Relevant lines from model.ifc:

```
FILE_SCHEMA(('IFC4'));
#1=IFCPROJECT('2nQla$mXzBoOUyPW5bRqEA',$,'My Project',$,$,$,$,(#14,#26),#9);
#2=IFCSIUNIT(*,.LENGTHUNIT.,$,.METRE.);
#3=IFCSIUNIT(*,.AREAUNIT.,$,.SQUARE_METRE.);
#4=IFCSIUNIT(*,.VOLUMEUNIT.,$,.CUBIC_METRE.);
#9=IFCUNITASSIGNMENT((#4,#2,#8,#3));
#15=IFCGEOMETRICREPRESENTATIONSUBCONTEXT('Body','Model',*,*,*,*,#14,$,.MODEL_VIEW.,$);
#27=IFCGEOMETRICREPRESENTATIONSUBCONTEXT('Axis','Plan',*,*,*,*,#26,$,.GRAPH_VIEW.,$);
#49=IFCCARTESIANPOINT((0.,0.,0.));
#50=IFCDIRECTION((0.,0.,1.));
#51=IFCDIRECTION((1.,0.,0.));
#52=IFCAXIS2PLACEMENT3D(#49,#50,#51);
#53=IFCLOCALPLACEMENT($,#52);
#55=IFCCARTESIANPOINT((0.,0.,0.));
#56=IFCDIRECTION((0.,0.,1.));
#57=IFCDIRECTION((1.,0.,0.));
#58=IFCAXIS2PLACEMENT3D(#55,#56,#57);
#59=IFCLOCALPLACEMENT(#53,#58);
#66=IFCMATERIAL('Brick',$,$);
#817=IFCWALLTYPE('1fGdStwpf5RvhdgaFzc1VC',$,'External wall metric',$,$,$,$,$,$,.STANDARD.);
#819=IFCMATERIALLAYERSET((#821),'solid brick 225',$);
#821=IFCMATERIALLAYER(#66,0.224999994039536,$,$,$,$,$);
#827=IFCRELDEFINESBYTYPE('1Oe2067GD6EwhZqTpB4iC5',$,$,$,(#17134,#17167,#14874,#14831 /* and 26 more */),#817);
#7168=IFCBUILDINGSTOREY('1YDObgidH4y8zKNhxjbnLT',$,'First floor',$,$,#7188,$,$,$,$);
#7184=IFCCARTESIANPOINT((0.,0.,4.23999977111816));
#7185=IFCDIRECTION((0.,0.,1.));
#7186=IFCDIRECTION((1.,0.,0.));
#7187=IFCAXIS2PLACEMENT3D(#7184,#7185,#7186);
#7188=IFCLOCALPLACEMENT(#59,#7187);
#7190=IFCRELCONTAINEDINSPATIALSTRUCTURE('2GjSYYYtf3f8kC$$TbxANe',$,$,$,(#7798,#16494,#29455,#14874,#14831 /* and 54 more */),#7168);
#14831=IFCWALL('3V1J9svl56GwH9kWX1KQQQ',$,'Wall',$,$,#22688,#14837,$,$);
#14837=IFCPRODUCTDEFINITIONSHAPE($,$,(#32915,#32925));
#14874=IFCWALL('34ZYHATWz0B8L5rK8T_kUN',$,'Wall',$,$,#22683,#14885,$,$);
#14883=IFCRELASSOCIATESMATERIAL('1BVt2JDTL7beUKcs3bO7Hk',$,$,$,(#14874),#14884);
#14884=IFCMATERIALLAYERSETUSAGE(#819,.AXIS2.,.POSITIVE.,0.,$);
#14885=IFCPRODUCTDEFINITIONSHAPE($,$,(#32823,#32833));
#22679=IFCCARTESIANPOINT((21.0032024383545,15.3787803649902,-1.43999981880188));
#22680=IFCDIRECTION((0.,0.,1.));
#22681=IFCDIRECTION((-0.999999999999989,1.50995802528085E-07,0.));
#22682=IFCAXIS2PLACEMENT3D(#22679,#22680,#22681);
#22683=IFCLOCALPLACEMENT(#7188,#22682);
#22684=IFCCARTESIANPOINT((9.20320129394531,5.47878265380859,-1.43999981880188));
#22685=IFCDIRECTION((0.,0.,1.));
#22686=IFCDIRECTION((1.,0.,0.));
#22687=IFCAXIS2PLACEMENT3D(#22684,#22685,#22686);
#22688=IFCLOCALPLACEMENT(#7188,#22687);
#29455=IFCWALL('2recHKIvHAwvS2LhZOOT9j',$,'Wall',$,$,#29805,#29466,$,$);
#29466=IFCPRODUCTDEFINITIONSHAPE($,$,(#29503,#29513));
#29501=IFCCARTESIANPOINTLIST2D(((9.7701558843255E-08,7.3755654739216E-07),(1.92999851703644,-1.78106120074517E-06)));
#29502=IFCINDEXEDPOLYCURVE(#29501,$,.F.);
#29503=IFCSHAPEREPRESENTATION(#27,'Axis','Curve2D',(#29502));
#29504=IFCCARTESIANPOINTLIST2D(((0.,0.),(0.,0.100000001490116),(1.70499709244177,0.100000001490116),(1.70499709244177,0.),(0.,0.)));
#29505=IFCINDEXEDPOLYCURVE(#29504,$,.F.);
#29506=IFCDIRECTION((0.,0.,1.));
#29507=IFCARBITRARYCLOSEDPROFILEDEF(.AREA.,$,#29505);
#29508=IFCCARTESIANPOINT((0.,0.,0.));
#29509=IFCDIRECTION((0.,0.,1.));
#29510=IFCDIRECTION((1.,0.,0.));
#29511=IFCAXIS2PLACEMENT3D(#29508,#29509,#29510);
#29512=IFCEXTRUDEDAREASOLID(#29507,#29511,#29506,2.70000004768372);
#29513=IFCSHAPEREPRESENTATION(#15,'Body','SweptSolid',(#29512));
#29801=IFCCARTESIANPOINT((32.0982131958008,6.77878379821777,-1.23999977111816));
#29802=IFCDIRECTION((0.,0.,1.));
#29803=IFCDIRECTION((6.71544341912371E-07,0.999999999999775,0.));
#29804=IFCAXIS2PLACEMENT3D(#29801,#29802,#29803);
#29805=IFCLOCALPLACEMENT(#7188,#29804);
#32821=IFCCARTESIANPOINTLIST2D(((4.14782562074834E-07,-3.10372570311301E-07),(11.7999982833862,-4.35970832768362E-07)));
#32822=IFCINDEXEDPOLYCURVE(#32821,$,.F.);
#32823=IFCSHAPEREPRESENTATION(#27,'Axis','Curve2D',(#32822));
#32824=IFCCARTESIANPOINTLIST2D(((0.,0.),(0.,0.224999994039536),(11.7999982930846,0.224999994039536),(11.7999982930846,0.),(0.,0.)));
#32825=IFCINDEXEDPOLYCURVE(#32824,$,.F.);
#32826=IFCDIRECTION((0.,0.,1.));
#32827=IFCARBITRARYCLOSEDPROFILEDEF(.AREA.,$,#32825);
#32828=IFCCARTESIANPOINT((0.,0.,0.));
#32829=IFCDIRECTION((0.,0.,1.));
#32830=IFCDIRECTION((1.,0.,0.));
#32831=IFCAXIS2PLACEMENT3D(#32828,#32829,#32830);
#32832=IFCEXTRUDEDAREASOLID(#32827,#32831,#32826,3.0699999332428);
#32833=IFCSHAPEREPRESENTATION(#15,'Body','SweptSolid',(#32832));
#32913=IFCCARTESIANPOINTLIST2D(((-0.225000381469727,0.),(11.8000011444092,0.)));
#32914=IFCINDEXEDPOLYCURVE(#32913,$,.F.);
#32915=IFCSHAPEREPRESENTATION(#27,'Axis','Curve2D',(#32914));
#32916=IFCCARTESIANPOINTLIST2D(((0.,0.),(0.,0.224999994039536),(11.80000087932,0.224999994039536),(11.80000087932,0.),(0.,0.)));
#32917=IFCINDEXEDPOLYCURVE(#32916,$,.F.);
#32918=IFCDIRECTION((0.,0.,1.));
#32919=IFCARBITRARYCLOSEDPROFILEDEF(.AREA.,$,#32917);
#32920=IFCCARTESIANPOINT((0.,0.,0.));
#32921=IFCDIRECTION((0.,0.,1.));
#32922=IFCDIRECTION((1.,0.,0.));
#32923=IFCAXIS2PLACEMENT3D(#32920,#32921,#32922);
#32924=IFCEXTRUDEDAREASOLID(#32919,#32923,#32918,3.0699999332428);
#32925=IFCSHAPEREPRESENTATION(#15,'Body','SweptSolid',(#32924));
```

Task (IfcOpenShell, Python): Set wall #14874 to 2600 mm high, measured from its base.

```python
import ifcopenshell
import ifcopenshell.geom
import ifcopenshell.util.representation
import ifcopenshell.util.shape

model = ifcopenshell.open("model.ifc")
settings = ifcopenshell.geom.settings()


def volume(element):
    """Net volume in cubic metres, openings subtracted."""
    shape = ifcopenshell.geom.create_shape(settings, element)
    return ifcopenshell.util.shape.get_volume(shape.geometry)


wall = model.by_guid("34ZYHATWz0B8L5rK8T_kUN")
before = volume(wall)

body = ifcopenshell.util.representation.get_representation(wall, "Model", "Body")
solid = body.Items[0]
old_height = solid.Depth
solid.Depth = 2.6
after = volume(wall)

print(f"height {old_height:g} -> {solid.Depth:g}, volume {before:.3f} -> {after:.3f} m3")

model.write("model-out.ifc")
```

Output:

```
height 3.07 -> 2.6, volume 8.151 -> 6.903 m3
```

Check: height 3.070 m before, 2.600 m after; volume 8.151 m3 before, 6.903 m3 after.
